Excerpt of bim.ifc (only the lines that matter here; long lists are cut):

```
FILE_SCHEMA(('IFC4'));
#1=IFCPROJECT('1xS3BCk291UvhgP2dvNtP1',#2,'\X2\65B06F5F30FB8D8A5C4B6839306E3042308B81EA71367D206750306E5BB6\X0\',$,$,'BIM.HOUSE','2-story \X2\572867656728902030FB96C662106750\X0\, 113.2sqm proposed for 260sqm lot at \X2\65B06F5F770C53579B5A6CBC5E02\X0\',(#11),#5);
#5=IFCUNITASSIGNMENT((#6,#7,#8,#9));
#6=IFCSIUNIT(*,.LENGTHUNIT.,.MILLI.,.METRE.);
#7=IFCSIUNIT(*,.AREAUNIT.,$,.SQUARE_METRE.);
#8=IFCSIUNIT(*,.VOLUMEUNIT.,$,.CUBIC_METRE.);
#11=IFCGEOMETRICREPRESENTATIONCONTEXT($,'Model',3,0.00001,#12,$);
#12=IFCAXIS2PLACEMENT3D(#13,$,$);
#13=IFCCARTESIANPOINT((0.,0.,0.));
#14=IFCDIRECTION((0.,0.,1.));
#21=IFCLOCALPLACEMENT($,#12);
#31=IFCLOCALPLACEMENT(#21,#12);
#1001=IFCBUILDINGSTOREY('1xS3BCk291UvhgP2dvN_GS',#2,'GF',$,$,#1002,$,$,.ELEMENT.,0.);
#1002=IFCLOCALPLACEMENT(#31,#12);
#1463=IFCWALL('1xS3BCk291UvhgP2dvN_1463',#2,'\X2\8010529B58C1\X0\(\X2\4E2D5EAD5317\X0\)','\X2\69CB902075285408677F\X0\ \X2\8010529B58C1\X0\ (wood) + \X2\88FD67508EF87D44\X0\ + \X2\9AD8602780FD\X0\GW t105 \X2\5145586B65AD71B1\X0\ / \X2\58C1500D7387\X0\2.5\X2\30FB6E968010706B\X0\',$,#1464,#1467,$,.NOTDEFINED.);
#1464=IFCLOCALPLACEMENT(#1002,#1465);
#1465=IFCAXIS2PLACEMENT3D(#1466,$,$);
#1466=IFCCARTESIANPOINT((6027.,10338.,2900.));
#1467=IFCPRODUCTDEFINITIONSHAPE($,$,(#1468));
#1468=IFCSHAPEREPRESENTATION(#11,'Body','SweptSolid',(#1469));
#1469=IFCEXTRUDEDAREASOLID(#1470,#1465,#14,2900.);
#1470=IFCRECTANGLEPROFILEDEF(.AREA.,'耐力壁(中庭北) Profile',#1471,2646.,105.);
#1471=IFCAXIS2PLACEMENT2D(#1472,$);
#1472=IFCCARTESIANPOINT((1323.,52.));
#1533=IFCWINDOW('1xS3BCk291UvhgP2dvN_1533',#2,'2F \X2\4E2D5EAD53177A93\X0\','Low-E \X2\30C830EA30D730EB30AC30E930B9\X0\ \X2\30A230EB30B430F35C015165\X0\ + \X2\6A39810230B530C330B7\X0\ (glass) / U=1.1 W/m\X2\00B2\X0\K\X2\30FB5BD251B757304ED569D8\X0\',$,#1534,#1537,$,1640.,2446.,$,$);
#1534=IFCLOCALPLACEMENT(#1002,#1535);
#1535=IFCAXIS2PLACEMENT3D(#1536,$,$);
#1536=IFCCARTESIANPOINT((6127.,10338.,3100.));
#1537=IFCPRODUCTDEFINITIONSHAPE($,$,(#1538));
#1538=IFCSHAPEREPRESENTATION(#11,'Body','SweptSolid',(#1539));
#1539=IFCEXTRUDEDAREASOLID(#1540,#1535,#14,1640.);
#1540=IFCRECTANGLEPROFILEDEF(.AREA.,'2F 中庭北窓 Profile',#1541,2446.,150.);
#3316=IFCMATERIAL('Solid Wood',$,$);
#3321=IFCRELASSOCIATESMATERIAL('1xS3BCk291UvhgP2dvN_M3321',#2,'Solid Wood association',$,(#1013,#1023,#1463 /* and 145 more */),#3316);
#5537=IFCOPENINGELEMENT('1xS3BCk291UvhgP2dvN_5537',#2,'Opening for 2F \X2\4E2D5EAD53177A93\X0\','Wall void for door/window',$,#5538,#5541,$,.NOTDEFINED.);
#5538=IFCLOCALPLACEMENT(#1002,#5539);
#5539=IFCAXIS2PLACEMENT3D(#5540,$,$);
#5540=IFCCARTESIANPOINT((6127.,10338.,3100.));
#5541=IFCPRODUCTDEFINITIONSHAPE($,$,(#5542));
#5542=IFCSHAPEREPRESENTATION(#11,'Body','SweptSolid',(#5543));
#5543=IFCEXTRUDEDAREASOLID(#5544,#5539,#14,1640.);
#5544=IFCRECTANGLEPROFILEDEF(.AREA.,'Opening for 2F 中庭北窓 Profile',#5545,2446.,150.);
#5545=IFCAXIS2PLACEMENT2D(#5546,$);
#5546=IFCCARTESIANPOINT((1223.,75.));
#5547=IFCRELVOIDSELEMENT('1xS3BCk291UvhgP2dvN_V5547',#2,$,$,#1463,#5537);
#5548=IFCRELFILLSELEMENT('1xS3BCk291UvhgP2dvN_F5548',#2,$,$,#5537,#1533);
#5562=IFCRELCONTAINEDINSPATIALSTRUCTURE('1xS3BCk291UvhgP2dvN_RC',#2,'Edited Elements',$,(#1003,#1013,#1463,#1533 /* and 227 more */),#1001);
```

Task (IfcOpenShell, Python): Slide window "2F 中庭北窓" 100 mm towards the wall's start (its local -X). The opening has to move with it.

```python
import ifcopenshell
import ifcopenshell.api.geometry
import ifcopenshell.util.placement
import ifcopenshell.util.unit

model = ifcopenshell.open("bim.ifc")
unit_scale = ifcopenshell.util.unit.calculate_unit_scale(model)

window = model.by_guid("1xS3BCk291UvhgP2dvN_1533")
opening = window.FillsVoids[0].RelatingOpeningElement
wall = opening.VoidsElements[0].RelatingBuildingElement

wall_matrix = ifcopenshell.util.placement.get_local_placement(wall.ObjectPlacement)
shift = wall_matrix[:3, 0] * -0.1 / unit_scale
before = ifcopenshell.util.placement.get_local_placement(window.ObjectPlacement)[:3, 3].copy()

# The window is not placed relative to its opening, so move both.
for product in (opening, window):
    matrix = ifcopenshell.util.placement.get_local_placement(product.ObjectPlacement)
    matrix[:3, 3] += shift
    ifcopenshell.api.geometry.edit_object_placement(model, product=product, matrix=matrix, is_si=False)

after = ifcopenshell.util.placement.get_local_placement(window.ObjectPlacement)[:3, 3]
print("window moved by", (after - before).round(3) + 0.0)

model.write("bim_v2.ifc")
```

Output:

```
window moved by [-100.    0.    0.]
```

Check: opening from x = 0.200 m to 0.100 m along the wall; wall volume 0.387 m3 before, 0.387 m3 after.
